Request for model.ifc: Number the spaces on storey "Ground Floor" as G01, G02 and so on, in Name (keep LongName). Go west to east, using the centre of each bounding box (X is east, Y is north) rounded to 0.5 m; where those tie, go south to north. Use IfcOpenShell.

First a look at what the model holds.

```python
import ifcopenshell
import ifcopenshell.util.element
import ifcopenshell.util.placement

model = ifcopenshell.open("model.ifc")
print(model.schema)
storey = next(s for s in model.by_type("IfcBuildingStorey") if s.Name == "Ground Floor")
spaces = [e for e in ifcopenshell.util.element.get_decomposition(storey) if e.is_a("IfcSpace")]
for e in sorted(spaces, key=lambda e: e.id()):
    origin = ifcopenshell.util.placement.get_local_placement(e.ObjectPlacement)[:3, 3]
    print(e.id(), e.Name, e.LongName, origin.round(2) + 0.0, sep=" | ")
```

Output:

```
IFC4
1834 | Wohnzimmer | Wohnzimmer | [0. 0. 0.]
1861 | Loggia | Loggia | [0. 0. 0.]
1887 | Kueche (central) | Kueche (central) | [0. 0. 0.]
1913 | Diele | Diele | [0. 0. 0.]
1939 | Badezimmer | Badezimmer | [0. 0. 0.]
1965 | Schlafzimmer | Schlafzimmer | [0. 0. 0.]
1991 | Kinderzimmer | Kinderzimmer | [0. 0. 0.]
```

```python
import ifcopenshell
import ifcopenshell.geom
import ifcopenshell.util.element
import ifcopenshell.util.shape

model = ifcopenshell.open("model.ifc")
settings = ifcopenshell.geom.settings()
settings.set("use-world-coords", True)


def centre(element):
    shape = ifcopenshell.geom.create_shape(settings, element)
    return ifcopenshell.util.shape.get_bbox_centroid(shape.geometry)


storey = next(s for s in model.by_type("IfcBuildingStorey") if s.Name == "Ground Floor")
spaces = [e for e in ifcopenshell.util.element.get_decomposition(storey) if e.is_a("IfcSpace")]

# Insertion points can sit at a corner or the storey origin, so sort by the geometry (in metres).
centres = {e: centre(e) for e in spaces}
spaces.sort(key=lambda e: (round(centres[e][0] / 0.5), centres[e][1]))

for i, e in enumerate(spaces, start=1):
    number = f"G{i:02d}"
    e.Name = number
    print(e.id(), number)

model.write("model_v2.ifc")
```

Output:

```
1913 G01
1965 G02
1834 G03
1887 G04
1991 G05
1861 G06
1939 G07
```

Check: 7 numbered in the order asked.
